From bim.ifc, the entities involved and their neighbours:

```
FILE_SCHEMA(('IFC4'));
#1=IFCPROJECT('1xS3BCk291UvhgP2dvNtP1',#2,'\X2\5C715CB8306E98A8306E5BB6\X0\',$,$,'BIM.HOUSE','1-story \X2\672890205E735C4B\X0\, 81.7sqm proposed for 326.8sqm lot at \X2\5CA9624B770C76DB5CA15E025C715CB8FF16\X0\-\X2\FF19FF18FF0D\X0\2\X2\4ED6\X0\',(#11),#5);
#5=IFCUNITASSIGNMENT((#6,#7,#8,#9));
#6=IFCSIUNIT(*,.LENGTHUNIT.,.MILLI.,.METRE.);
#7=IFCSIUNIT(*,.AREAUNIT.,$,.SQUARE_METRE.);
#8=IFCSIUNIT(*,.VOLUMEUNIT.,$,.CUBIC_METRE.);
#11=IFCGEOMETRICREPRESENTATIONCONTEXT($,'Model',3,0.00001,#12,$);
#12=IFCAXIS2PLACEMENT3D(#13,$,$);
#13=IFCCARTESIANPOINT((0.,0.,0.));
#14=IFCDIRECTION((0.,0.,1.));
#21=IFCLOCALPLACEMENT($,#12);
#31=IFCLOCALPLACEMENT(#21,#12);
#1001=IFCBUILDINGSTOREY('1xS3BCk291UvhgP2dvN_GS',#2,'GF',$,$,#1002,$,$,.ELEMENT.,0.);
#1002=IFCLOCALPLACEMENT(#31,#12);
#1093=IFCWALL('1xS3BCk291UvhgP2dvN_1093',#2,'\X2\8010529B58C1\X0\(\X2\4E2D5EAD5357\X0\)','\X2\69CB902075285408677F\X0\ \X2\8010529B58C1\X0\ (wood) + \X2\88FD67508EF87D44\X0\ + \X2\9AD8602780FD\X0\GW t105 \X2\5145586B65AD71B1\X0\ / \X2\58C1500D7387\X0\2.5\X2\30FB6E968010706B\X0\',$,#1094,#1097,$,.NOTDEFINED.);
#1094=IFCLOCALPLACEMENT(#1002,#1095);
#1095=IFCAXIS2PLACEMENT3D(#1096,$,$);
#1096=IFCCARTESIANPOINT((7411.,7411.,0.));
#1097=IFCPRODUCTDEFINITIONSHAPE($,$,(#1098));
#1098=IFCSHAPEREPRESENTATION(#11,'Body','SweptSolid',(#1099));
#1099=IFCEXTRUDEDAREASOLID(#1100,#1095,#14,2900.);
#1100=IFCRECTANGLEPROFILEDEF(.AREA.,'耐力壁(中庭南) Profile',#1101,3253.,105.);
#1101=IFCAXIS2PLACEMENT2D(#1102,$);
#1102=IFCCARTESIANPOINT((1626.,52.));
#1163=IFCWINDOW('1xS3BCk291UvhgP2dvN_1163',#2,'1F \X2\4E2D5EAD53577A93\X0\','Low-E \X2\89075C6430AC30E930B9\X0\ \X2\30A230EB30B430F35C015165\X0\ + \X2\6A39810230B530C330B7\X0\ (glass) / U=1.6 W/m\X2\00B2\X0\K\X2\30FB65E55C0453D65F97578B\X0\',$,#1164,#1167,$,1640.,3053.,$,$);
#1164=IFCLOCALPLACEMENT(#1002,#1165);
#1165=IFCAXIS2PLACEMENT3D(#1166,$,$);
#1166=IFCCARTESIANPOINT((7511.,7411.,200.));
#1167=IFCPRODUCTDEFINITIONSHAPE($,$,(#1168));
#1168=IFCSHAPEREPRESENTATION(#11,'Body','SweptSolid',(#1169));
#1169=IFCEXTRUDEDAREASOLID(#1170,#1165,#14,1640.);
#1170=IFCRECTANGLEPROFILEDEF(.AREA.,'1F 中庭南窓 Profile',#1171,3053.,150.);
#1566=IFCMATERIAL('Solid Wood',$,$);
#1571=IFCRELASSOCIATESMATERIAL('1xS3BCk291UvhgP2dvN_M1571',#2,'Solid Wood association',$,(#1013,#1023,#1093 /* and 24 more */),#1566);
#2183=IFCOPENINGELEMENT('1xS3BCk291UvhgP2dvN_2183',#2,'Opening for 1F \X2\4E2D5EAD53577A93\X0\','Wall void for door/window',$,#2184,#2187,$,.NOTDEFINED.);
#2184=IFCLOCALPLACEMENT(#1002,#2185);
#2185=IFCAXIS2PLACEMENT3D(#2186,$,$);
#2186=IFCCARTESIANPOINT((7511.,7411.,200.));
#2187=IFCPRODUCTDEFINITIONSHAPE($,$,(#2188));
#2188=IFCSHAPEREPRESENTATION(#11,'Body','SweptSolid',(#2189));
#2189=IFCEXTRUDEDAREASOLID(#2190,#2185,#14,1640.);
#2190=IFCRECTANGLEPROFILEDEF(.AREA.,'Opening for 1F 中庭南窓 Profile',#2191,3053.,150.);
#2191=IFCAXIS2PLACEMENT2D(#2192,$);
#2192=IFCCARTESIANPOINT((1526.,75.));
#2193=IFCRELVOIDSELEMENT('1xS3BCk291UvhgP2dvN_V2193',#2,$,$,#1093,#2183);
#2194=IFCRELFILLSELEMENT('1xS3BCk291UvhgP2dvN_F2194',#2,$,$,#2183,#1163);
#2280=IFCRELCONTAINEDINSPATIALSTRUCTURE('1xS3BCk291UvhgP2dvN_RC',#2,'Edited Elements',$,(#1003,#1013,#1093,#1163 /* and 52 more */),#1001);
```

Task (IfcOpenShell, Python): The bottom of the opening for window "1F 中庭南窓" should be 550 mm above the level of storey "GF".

```python
import numpy as np
import ifcopenshell
import ifcopenshell.api.geometry
import ifcopenshell.geom
import ifcopenshell.util.element
import ifcopenshell.util.placement
import ifcopenshell.util.shape
import ifcopenshell.util.unit

model = ifcopenshell.open("bim.ifc")
unit_scale = ifcopenshell.util.unit.calculate_unit_scale(model)

window = model.by_guid("1xS3BCk291UvhgP2dvN_1163")
opening = window.FillsVoids[0].RelatingOpeningElement
storey = ifcopenshell.util.element.get_container(window, ifc_class="IfcBuildingStorey")
level = ifcopenshell.util.placement.get_local_placement(storey.ObjectPlacement)[2, 3]

# The opening's origin need not be at the sill, so measure its lowest point.
shape = ifcopenshell.geom.create_shape(ifcopenshell.geom.settings(), opening)
bottom = ifcopenshell.util.shape.get_shape_bottom_elevation(shape, shape.geometry) / unit_scale
dz = level + 550.0 - bottom

shift = np.array([0.0, 0.0, dz])
# The window is not placed relative to its opening, so move both.
for product in (opening, window):
    matrix = ifcopenshell.util.placement.get_local_placement(product.ObjectPlacement)
    matrix[:3, 3] += shift
    ifcopenshell.api.geometry.edit_object_placement(model, product=product, matrix=matrix, is_si=False)

print(f"moved by {dz * unit_scale:+.3f} m")

model.write("bim_updated.ifc")
```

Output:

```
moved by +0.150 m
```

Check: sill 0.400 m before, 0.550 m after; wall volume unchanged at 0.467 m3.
